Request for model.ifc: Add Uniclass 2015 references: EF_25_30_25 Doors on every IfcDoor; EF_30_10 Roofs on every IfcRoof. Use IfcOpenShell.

First a look at what the model holds.

```python
import ifcopenshell

model = ifcopenshell.open("model.ifc")
print(model.schema)
print("classifications:", [c.Name for c in model.by_type("IfcClassification")])
for ifc_class in ("IfcDoor", "IfcRoof", "IfcStair", "IfcWall", "IfcWindow"):
    print(ifc_class, len(model.by_type(ifc_class)))
```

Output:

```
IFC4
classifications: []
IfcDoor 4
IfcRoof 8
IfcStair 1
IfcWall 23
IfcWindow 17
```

```python
import ifcopenshell
import ifcopenshell.api.classification

model = ifcopenshell.open("model.ifc")

system = ifcopenshell.api.classification.add_classification(model, classification="Uniclass 2015")

codes = {
    "IfcDoor": ("EF_25_30_25", "Doors"),
    "IfcRoof": ("EF_30_10", "Roofs"),
}
for ifc_class, (code, name) in codes.items():
    products = model.by_type(ifc_class)
    ifcopenshell.api.classification.add_reference(
        model, products=products, classification=system, identification=code, name=name
    )
    print(code, len(products))

model.write("model-out.ifc")
```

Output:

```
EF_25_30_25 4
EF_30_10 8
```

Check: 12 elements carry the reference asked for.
